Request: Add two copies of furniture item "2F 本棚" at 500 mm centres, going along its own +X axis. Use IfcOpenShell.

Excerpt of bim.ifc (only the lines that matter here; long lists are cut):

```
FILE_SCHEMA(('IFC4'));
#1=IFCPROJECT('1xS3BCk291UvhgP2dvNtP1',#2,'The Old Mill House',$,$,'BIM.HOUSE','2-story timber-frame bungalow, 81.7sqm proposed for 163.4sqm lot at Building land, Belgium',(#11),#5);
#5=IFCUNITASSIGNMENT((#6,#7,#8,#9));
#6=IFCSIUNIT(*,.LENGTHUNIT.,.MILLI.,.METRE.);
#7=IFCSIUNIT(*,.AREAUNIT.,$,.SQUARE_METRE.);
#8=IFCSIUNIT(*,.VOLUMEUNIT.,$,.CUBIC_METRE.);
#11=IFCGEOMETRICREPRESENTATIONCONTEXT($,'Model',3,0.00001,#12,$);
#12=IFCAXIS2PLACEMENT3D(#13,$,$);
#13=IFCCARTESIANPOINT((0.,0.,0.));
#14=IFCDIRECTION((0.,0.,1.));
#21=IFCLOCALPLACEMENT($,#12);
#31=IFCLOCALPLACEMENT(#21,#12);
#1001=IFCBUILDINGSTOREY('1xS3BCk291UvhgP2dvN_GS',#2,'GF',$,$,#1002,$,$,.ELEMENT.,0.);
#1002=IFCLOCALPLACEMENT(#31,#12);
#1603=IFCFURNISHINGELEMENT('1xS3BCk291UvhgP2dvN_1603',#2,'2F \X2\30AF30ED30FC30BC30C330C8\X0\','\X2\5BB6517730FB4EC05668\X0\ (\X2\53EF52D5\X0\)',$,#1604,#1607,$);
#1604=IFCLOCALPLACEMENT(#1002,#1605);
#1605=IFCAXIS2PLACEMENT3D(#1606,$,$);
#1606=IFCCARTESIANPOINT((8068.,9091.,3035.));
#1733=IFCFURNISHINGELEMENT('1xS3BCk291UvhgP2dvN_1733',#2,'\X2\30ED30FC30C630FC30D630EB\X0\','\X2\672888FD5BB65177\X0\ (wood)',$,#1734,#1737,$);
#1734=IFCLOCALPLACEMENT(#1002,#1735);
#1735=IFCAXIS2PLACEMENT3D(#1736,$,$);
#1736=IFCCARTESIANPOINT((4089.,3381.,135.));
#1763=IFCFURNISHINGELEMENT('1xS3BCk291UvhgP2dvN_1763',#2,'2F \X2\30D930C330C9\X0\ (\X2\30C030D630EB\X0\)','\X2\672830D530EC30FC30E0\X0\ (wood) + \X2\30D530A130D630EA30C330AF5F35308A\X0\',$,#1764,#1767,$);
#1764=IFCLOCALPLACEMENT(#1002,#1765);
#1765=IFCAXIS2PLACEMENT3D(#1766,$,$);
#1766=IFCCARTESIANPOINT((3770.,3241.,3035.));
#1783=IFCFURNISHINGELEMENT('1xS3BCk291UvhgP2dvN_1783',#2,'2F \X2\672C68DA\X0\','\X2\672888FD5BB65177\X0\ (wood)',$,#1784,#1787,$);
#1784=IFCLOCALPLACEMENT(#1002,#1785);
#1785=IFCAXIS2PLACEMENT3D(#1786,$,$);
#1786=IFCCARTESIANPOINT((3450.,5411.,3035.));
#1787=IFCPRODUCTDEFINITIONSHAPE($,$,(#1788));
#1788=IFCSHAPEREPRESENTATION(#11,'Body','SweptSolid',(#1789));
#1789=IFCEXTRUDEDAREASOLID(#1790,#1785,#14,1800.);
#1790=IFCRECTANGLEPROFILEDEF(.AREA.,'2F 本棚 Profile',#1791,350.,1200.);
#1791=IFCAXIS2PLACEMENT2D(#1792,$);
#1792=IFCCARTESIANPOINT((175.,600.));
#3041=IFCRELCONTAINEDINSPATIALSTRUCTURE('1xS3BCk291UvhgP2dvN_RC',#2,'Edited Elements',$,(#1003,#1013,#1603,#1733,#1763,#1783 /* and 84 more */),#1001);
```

```python
import ifcopenshell
import ifcopenshell.api.geometry
import ifcopenshell.api.root
import ifcopenshell.util.element
import ifcopenshell.util.placement

model = ifcopenshell.open("bim.ifc")


def reuse_history(source, copy):
    """copy_class also copies each property set's owner history, people and application; keep the originals."""
    for rel in copy.IsDefinedBy:
        if rel.is_a("IfcRelDefinesByProperties") and (history := rel.RelatingPropertyDefinition.OwnerHistory):
            rel.RelatingPropertyDefinition.OwnerHistory = source.OwnerHistory
            ifcopenshell.util.element.remove_deep2(model, history)


source = model.by_guid("1xS3BCk291UvhgP2dvN_1783")
base = ifcopenshell.util.placement.get_local_placement(source.ObjectPlacement)
step = base[:3, 0] * 500.0

for i in range(1, 3):
    copy = ifcopenshell.api.root.copy_class(model, product=source)
    copy.Representation = ifcopenshell.util.element.copy_deep(
        model, source.Representation, exclude=["IfcGeometricRepresentationContext", "IfcRepresentationMap"]
    )
    reuse_history(source, copy)
    matrix = base.copy()
    matrix[:3, 3] += i * step
    print("added at", matrix[:3, 3].round(3) + 0.0)
    ifcopenshell.api.geometry.edit_object_placement(model, product=copy, matrix=matrix, is_si=False)

model.write("bim_v2.ifc")
```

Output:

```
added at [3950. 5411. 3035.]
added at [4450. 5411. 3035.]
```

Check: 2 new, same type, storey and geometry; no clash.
